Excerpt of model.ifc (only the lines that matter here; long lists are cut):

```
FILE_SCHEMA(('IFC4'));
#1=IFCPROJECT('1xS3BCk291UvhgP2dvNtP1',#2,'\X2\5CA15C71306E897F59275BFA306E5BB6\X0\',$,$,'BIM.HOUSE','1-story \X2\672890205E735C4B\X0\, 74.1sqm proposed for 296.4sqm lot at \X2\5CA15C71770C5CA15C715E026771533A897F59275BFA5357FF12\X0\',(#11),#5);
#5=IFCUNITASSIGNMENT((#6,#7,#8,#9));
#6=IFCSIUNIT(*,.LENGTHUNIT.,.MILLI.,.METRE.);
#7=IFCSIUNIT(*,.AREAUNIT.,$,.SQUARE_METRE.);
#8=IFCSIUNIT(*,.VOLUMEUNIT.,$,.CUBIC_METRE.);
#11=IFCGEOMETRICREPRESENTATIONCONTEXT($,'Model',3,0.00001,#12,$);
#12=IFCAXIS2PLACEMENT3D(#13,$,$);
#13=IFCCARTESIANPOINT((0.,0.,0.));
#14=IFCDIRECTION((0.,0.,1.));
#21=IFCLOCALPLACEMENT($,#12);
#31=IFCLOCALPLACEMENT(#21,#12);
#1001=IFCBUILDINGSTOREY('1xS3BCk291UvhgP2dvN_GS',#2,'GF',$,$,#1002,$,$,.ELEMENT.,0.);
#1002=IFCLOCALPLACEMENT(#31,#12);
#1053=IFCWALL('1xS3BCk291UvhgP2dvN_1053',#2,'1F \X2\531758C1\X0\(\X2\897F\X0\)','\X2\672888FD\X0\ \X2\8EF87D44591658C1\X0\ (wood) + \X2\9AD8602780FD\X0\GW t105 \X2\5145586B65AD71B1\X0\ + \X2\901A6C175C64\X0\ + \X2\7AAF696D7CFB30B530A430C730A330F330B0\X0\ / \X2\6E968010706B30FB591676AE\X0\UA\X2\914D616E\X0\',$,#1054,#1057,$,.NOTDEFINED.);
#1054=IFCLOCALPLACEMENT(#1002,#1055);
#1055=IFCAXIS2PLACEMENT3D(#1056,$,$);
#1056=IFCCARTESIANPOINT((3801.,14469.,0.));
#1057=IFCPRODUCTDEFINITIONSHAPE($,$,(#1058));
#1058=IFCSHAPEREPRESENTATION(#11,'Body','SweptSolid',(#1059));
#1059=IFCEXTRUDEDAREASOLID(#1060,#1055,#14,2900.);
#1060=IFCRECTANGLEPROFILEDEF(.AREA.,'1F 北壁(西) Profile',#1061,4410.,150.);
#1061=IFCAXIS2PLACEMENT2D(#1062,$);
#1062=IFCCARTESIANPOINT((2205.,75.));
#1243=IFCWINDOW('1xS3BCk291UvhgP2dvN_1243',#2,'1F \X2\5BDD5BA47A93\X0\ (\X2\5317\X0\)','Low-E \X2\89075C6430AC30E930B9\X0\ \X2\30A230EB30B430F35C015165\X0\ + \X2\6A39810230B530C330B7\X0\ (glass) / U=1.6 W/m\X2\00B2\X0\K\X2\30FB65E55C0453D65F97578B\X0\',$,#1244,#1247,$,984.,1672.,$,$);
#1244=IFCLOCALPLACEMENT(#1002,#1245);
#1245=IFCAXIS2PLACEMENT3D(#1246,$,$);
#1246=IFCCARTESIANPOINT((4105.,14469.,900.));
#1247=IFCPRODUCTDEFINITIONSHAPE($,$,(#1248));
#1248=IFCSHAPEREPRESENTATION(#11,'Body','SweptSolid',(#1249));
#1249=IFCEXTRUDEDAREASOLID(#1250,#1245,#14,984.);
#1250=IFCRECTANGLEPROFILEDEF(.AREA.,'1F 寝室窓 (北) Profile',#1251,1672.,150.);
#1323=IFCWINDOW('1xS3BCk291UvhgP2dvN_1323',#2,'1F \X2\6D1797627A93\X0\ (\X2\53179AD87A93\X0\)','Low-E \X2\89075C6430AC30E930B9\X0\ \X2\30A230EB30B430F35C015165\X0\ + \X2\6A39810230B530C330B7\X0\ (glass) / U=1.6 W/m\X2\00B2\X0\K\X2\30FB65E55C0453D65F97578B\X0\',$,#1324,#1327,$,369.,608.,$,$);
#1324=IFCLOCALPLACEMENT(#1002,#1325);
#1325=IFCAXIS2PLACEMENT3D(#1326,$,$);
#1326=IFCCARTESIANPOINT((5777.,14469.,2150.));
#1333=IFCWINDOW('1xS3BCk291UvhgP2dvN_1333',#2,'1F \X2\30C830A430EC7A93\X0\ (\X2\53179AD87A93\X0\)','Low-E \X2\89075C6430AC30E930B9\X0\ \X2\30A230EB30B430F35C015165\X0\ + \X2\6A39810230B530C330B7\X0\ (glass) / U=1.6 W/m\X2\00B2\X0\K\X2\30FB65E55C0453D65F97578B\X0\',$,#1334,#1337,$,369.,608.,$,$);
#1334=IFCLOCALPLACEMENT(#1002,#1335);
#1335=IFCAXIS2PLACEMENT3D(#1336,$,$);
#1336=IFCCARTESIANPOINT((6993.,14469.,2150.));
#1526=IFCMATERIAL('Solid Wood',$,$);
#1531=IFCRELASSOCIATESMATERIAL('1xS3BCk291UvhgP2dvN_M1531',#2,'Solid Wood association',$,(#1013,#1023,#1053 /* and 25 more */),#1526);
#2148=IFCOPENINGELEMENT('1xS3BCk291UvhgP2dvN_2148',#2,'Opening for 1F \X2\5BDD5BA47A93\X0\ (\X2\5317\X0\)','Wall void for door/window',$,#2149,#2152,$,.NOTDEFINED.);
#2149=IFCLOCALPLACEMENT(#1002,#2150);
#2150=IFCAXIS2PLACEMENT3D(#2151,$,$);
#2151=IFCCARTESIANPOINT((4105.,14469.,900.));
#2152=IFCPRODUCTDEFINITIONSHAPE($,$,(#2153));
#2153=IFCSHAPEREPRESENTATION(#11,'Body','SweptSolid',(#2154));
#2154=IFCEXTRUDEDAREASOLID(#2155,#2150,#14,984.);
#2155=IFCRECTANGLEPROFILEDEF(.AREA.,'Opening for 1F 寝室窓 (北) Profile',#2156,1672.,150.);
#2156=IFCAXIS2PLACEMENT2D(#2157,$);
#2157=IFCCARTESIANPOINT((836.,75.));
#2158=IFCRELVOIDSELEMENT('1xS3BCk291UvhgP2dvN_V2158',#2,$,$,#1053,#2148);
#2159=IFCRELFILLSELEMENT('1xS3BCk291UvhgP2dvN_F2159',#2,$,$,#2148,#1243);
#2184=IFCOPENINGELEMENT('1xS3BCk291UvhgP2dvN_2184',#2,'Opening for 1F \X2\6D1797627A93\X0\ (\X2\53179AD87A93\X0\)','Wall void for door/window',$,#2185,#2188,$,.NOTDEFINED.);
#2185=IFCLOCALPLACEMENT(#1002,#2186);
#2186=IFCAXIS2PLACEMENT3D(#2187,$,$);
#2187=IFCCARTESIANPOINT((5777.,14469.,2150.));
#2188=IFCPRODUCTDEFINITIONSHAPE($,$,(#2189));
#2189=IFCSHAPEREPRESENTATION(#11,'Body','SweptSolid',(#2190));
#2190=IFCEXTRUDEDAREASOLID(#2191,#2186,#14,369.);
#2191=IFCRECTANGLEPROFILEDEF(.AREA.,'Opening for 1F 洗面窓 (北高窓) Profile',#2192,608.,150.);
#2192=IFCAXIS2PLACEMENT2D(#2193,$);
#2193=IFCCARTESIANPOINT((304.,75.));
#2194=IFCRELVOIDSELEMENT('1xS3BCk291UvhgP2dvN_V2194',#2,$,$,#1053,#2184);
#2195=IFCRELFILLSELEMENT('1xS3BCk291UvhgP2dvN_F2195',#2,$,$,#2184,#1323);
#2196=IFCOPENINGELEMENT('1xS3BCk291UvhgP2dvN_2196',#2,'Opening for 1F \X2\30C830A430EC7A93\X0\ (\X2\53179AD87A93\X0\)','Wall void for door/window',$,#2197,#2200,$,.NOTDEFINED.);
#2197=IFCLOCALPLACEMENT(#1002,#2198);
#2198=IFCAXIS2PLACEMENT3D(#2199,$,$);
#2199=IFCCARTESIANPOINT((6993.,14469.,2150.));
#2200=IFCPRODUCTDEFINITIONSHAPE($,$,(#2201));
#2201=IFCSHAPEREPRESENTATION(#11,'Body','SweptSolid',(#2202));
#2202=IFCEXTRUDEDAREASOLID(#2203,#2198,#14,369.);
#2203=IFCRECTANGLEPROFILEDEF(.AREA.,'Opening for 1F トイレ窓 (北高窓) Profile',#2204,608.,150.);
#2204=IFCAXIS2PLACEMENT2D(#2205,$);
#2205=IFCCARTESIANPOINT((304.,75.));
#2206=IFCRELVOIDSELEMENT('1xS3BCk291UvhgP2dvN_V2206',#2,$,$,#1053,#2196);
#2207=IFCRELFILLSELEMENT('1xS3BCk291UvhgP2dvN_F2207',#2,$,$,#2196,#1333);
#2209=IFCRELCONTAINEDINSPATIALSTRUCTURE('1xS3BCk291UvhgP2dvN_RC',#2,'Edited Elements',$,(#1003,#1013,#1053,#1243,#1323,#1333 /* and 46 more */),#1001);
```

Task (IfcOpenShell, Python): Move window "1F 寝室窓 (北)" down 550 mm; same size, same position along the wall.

```python
import numpy as np
import ifcopenshell
import ifcopenshell.api.geometry
import ifcopenshell.util.placement
import ifcopenshell.util.unit

model = ifcopenshell.open("model.ifc")
unit_scale = ifcopenshell.util.unit.calculate_unit_scale(model)

window = model.by_guid("1xS3BCk291UvhgP2dvN_1243")
opening = window.FillsVoids[0].RelatingOpeningElement
dz = -550.0

shift = np.array([0.0, 0.0, dz])
# The window is not placed relative to its opening, so move both.
for product in (opening, window):
    matrix = ifcopenshell.util.placement.get_local_placement(product.ObjectPlacement)
    matrix[:3, 3] += shift
    ifcopenshell.api.geometry.edit_object_placement(model, product=product, matrix=matrix, is_si=False)

print(f"moved by {dz * unit_scale:+.3f} m")

model.write("model_updated.ifc")
```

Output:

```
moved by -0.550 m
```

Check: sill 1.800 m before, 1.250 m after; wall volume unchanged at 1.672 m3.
